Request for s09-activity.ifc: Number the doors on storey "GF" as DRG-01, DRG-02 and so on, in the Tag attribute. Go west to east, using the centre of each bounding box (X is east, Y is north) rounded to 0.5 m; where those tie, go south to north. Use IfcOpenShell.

First a look at what the model holds.

```python
import ifcopenshell
import ifcopenshell.util.element
import ifcopenshell.util.placement

model = ifcopenshell.open("s09-activity.ifc")
print(model.schema)
storey = next(s for s in model.by_type("IfcBuildingStorey") if s.Name == "GF")
doors = [e for e in ifcopenshell.util.element.get_decomposition(storey) if e.is_a("IfcDoor")]
for e in sorted(doors, key=lambda e: e.id()):
    origin = ifcopenshell.util.placement.get_local_placement(e.ObjectPlacement)[:3, 3]
    print(e.id(), e.Tag, e.Name, origin.round(2) + 0.0, sep=" | ")
```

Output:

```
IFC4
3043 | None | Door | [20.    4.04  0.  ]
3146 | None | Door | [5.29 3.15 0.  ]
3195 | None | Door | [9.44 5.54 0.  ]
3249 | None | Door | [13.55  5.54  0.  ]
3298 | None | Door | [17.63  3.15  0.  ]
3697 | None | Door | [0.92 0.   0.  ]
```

```python
import ifcopenshell
import ifcopenshell.geom
import ifcopenshell.util.element
import ifcopenshell.util.shape

model = ifcopenshell.open("s09-activity.ifc")
settings = ifcopenshell.geom.settings()
settings.set("use-world-coords", True)


def centre(element):
    shape = ifcopenshell.geom.create_shape(settings, element)
    return ifcopenshell.util.shape.get_bbox_centroid(shape.geometry)


storey = next(s for s in model.by_type("IfcBuildingStorey") if s.Name == "GF")
doors = [e for e in ifcopenshell.util.element.get_decomposition(storey) if e.is_a("IfcDoor")]

# Insertion points can sit at a corner or the storey origin, so sort by the geometry (in metres).
centres = {e: centre(e) for e in doors}
doors.sort(key=lambda e: (round(centres[e][0] / 0.5), centres[e][1]))

for i, e in enumerate(doors, start=1):
    number = f"DRG-{i:02d}"
    e.Tag = number
    print(e.id(), number)

model.write("s09-activity-out.ifc")
```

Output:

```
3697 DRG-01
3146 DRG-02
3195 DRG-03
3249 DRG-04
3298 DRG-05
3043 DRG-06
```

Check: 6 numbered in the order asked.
